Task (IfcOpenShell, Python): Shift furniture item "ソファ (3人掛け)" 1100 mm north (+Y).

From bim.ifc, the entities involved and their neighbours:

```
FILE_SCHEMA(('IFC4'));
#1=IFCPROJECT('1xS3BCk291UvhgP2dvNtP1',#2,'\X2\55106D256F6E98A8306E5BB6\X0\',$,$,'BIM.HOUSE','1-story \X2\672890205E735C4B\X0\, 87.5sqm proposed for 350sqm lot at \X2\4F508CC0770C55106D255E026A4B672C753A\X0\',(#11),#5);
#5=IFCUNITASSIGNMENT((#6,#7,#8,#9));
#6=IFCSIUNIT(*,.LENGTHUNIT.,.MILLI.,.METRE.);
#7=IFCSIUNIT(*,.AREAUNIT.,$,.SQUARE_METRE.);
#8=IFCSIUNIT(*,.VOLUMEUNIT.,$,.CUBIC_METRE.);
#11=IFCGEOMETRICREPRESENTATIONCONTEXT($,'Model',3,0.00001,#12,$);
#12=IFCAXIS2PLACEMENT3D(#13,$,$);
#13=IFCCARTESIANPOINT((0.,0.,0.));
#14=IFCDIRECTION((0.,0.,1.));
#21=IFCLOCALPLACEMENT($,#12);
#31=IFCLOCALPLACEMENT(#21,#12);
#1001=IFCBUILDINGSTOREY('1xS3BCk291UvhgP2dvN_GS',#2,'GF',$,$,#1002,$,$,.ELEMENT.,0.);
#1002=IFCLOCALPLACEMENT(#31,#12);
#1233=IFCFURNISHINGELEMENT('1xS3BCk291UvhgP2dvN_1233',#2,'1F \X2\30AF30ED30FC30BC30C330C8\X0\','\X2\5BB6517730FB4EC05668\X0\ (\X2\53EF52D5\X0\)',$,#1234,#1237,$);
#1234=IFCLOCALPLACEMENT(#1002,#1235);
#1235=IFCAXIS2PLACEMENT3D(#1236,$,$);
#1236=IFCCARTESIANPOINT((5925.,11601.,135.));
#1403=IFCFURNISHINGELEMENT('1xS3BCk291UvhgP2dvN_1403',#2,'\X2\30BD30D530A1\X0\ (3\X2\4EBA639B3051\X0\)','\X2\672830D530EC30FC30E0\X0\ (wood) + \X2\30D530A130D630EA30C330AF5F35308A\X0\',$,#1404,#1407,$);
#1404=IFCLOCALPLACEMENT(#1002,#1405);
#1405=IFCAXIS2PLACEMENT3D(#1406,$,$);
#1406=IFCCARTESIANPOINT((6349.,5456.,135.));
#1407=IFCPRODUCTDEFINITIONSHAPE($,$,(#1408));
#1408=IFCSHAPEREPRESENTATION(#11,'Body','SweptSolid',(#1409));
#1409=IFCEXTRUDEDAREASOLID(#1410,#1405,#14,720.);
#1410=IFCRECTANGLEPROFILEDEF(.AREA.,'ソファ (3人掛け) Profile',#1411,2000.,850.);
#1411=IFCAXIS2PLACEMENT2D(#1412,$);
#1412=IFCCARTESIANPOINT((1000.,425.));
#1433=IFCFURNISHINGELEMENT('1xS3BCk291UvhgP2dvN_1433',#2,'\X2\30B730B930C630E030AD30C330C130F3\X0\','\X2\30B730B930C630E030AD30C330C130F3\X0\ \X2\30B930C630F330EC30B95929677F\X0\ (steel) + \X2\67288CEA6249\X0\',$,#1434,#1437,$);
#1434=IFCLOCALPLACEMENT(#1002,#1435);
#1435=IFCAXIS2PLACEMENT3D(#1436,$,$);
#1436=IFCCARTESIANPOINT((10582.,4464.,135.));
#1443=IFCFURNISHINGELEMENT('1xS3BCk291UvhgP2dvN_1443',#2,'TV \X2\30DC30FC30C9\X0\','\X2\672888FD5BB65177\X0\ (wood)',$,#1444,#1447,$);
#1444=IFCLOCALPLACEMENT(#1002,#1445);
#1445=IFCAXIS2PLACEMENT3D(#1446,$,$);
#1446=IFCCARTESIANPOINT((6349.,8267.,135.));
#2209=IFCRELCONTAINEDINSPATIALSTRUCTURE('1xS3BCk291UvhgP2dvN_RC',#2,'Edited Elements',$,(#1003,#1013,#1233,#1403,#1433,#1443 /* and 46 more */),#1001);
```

```python
import ifcopenshell
import ifcopenshell.api.geometry
import ifcopenshell.util.placement

model = ifcopenshell.open("bim.ifc")

item = model.by_id(1403)
matrix = ifcopenshell.util.placement.get_local_placement(item.ObjectPlacement)
matrix[1, 3] += 1100.0
ifcopenshell.api.geometry.edit_object_placement(model, product=item, matrix=matrix, is_si=False)

print(ifcopenshell.util.placement.get_local_placement(item.ObjectPlacement).round(3) + 0.0)

model.write("bim_edited.ifc")
```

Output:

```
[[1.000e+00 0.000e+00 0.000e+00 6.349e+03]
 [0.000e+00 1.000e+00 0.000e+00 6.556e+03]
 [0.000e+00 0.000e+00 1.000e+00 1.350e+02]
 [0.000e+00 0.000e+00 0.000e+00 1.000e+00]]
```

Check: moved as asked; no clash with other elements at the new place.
